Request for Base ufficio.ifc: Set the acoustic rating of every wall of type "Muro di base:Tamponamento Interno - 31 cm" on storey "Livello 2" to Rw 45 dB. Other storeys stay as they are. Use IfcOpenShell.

First a look at what the model holds.

```python
import ifcopenshell
import ifcopenshell.util.element

model = ifcopenshell.open("Base ufficio.ifc")
print(model.schema)
storey = next(s for s in model.by_type("IfcBuildingStorey") if s.Name == "Livello 2")
walls = [e for e in ifcopenshell.util.element.get_decomposition(storey) if e.is_a("IfcWall")]
seen = {}
for e in walls:
    element_type = ifcopenshell.util.element.get_type(e)
    key = (element_type.Name if element_type != e and element_type else None, ifcopenshell.util.element.get_pset(e, "Pset_WallCommon", "AcousticRating"))
    seen[key] = seen.get(key, 0) + 1
for (name, value), count in sorted(seen.items(), key=str):
    print(count, "x", name, "|", value)
```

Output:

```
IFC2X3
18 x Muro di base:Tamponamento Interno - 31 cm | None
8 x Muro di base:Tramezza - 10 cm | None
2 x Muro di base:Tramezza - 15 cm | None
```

```python
import ifcopenshell
import ifcopenshell.api.pset
import ifcopenshell.util.element

model = ifcopenshell.open("Base ufficio.ifc")

storey = next(s for s in model.by_type("IfcBuildingStorey") if s.Name == "Livello 2")
walls = [e for e in ifcopenshell.util.element.get_decomposition(storey) if e.is_a("IfcWall")]

count = 0
for e in walls:
    element_type = ifcopenshell.util.element.get_type(e)
    if element_type in (None, e) or element_type.Name != "Muro di base:Tamponamento Interno - 31 cm":
        continue
    # add_pset returns the element's existing set when there is one.
    pset = ifcopenshell.api.pset.add_pset(model, product=e, name="Pset_WallCommon")
    ifcopenshell.api.pset.edit_pset(model, pset=pset, properties={"AcousticRating": "Rw 45 dB"})
    count += 1

print(count, "walls updated")

model.write("Base ufficio_v2.ifc")
```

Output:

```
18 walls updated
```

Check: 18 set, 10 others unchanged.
